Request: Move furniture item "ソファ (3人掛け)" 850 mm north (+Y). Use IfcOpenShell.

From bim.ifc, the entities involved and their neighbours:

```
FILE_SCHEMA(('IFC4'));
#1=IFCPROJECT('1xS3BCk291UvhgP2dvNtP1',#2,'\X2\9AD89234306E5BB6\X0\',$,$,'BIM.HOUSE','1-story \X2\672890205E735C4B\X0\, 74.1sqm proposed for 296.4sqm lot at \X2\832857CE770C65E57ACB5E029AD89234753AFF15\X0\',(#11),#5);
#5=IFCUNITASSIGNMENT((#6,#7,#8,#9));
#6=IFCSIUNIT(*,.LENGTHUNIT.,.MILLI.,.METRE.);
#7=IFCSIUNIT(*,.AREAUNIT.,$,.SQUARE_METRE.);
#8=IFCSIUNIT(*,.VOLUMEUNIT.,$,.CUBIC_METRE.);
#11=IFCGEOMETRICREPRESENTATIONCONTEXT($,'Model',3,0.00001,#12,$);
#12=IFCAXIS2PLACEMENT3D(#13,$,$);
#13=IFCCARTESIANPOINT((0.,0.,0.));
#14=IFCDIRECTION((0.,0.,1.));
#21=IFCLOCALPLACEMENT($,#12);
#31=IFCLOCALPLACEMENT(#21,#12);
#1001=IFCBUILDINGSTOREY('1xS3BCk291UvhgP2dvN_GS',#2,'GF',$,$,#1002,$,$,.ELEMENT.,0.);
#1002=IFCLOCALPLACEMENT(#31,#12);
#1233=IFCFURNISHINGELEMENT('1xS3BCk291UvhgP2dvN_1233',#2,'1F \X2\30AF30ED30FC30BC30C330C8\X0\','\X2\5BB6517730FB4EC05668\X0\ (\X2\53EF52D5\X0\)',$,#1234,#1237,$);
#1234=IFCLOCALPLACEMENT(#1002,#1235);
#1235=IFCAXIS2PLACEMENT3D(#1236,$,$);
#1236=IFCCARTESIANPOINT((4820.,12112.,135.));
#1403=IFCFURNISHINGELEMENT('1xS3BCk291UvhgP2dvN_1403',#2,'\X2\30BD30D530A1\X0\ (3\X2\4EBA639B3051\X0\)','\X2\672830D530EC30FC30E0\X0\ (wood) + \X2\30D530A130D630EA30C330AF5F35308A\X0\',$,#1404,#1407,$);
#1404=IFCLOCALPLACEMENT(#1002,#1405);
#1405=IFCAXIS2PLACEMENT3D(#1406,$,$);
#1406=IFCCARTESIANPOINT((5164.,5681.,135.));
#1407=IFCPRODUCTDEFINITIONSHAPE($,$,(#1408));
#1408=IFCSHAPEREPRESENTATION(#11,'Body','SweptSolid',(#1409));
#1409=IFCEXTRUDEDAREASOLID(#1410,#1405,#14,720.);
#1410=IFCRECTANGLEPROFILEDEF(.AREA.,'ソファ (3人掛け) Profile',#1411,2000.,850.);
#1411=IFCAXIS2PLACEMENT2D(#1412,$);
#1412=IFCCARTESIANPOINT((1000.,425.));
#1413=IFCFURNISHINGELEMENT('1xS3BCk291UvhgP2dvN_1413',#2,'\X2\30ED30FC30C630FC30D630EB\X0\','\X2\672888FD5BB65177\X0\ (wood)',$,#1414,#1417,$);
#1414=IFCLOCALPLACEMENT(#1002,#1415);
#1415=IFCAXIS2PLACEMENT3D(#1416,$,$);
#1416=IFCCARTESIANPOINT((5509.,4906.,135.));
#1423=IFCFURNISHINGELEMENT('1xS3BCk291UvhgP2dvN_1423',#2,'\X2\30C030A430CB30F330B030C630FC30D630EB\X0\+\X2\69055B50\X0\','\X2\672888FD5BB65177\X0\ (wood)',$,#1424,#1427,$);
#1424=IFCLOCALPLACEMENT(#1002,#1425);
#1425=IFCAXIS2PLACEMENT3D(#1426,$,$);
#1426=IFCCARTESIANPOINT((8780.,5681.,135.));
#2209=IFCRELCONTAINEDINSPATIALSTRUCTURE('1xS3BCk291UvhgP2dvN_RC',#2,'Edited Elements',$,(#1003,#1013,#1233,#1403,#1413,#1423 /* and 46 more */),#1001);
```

```python
import ifcopenshell
import ifcopenshell.api.geometry
import ifcopenshell.util.placement
import ifcopenshell.util.unit

model = ifcopenshell.open("bim.ifc")
unit_scale = ifcopenshell.util.unit.calculate_unit_scale(model)

item = model.by_guid("1xS3BCk291UvhgP2dvN_1403")
matrix = ifcopenshell.util.placement.get_local_placement(item.ObjectPlacement)
matrix[1, 3] += 0.85 / unit_scale
ifcopenshell.api.geometry.edit_object_placement(model, product=item, matrix=matrix, is_si=False)

print(ifcopenshell.util.placement.get_local_placement(item.ObjectPlacement).round(3) + 0.0)

model.write("bim_updated.ifc")
```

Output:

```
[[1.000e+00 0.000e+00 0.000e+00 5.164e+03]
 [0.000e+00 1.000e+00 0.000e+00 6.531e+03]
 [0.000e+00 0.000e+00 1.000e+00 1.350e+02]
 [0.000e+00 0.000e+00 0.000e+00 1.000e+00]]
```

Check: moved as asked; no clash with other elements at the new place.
